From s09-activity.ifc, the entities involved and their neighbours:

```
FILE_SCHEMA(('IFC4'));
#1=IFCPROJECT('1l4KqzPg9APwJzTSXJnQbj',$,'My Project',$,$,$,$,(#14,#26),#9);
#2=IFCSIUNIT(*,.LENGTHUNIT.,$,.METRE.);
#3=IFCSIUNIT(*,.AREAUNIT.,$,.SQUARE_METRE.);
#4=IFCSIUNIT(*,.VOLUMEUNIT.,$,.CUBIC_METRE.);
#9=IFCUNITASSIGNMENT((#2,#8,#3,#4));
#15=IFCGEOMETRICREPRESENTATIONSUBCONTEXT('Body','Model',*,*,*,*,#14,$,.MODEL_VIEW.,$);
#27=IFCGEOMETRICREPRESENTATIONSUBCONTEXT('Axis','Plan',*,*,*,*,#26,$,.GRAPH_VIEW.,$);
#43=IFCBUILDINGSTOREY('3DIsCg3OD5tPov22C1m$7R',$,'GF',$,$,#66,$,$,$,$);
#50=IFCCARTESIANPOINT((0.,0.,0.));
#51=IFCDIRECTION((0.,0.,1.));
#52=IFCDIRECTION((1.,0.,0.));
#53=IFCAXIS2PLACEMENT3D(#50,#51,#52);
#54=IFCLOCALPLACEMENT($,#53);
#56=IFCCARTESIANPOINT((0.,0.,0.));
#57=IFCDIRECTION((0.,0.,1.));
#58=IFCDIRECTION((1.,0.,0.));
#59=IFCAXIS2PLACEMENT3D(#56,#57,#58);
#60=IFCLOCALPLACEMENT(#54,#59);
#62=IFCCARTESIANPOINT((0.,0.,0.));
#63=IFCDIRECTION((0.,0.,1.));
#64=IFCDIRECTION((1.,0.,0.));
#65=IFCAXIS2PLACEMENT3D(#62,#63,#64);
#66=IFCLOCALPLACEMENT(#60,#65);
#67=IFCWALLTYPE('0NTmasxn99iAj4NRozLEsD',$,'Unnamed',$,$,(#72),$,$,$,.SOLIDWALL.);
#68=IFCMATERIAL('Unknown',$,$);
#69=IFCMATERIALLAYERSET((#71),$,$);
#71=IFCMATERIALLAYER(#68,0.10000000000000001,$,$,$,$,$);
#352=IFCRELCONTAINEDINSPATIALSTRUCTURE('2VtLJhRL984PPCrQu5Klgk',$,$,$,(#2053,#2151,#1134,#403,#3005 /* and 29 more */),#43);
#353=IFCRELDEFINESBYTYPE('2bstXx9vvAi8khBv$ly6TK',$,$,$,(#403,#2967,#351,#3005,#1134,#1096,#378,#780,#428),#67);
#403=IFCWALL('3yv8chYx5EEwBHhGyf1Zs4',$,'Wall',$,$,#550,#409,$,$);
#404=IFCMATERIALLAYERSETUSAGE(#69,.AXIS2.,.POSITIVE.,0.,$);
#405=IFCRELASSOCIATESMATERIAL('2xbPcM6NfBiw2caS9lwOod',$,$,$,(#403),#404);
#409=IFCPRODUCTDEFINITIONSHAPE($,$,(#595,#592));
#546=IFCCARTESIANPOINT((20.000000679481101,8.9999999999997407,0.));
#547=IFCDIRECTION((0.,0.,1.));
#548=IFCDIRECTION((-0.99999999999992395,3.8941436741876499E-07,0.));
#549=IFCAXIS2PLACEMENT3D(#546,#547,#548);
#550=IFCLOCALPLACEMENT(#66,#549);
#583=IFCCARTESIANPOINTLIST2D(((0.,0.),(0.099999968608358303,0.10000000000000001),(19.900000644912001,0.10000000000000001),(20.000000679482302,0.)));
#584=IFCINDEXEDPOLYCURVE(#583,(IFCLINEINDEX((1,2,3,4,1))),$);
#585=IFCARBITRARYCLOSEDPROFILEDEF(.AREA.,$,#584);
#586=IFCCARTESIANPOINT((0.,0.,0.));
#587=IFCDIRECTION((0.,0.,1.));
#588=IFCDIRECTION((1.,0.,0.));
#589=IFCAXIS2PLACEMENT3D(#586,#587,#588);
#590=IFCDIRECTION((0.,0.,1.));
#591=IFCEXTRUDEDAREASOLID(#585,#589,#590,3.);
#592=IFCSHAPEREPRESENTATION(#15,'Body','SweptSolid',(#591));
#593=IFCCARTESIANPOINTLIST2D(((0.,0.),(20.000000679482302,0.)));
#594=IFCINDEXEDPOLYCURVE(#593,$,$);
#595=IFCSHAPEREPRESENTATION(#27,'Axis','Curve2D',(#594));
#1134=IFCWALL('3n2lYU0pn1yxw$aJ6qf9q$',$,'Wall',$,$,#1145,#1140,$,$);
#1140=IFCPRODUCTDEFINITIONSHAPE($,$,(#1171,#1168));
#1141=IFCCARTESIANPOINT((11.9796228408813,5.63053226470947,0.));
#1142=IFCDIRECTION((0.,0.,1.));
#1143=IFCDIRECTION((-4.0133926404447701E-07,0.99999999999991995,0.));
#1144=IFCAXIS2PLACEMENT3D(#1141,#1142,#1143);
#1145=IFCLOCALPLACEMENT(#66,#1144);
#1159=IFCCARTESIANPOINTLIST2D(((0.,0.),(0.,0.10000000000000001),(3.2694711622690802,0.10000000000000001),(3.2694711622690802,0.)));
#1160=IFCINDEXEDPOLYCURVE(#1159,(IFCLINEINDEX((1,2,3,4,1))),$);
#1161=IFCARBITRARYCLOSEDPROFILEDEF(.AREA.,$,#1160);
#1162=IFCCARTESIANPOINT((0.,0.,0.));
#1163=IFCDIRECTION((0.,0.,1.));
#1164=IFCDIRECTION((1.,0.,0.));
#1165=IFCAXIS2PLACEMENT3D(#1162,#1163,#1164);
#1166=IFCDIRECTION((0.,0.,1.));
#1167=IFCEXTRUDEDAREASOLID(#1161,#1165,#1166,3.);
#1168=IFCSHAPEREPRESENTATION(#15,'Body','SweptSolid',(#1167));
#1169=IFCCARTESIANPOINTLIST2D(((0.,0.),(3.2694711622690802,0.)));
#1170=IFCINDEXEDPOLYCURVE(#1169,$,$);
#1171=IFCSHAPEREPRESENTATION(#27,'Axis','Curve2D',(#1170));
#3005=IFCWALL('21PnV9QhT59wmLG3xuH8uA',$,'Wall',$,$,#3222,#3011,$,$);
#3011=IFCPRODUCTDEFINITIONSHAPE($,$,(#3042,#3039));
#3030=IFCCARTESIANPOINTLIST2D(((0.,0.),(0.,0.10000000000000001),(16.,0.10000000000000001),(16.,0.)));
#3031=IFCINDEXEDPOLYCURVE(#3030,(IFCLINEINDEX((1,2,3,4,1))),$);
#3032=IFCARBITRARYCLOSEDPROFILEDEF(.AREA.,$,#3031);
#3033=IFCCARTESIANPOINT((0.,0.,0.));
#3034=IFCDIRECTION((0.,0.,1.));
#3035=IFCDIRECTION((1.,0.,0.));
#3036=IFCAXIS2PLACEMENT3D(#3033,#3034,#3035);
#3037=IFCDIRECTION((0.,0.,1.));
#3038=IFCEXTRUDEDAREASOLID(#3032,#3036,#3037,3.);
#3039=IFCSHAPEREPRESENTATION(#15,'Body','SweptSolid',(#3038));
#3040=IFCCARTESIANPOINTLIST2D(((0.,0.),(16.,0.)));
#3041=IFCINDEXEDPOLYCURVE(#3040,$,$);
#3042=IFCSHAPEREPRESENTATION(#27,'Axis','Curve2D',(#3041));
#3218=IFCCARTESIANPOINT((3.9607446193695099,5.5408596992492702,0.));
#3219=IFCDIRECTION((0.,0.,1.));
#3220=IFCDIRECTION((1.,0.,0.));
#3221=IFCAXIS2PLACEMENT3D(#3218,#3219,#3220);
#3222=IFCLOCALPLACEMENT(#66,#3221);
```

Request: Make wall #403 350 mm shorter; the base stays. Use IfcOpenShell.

```python
import ifcopenshell
import ifcopenshell.geom
import ifcopenshell.util.representation
import ifcopenshell.util.shape
import ifcopenshell.util.unit

model = ifcopenshell.open("s09-activity.ifc")
unit_scale = ifcopenshell.util.unit.calculate_unit_scale(model)
settings = ifcopenshell.geom.settings()


def volume(element):
    """Net volume in cubic metres, openings subtracted."""
    shape = ifcopenshell.geom.create_shape(settings, element)
    return ifcopenshell.util.shape.get_volume(shape.geometry)


wall = model.by_guid("3yv8chYx5EEwBHhGyf1Zs4")
before = volume(wall)

body = ifcopenshell.util.representation.get_representation(wall, "Model", "Body")
solid = body.Items[0]
old_height = solid.Depth
solid.Depth -= 0.35 / unit_scale
after = volume(wall)

print(f"height {old_height:g} -> {solid.Depth:g}, volume {before:.3f} -> {after:.3f} m3")

model.write("s09-activity_updated.ifc")
```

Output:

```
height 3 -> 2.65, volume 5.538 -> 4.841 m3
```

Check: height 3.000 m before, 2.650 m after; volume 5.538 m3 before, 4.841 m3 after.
